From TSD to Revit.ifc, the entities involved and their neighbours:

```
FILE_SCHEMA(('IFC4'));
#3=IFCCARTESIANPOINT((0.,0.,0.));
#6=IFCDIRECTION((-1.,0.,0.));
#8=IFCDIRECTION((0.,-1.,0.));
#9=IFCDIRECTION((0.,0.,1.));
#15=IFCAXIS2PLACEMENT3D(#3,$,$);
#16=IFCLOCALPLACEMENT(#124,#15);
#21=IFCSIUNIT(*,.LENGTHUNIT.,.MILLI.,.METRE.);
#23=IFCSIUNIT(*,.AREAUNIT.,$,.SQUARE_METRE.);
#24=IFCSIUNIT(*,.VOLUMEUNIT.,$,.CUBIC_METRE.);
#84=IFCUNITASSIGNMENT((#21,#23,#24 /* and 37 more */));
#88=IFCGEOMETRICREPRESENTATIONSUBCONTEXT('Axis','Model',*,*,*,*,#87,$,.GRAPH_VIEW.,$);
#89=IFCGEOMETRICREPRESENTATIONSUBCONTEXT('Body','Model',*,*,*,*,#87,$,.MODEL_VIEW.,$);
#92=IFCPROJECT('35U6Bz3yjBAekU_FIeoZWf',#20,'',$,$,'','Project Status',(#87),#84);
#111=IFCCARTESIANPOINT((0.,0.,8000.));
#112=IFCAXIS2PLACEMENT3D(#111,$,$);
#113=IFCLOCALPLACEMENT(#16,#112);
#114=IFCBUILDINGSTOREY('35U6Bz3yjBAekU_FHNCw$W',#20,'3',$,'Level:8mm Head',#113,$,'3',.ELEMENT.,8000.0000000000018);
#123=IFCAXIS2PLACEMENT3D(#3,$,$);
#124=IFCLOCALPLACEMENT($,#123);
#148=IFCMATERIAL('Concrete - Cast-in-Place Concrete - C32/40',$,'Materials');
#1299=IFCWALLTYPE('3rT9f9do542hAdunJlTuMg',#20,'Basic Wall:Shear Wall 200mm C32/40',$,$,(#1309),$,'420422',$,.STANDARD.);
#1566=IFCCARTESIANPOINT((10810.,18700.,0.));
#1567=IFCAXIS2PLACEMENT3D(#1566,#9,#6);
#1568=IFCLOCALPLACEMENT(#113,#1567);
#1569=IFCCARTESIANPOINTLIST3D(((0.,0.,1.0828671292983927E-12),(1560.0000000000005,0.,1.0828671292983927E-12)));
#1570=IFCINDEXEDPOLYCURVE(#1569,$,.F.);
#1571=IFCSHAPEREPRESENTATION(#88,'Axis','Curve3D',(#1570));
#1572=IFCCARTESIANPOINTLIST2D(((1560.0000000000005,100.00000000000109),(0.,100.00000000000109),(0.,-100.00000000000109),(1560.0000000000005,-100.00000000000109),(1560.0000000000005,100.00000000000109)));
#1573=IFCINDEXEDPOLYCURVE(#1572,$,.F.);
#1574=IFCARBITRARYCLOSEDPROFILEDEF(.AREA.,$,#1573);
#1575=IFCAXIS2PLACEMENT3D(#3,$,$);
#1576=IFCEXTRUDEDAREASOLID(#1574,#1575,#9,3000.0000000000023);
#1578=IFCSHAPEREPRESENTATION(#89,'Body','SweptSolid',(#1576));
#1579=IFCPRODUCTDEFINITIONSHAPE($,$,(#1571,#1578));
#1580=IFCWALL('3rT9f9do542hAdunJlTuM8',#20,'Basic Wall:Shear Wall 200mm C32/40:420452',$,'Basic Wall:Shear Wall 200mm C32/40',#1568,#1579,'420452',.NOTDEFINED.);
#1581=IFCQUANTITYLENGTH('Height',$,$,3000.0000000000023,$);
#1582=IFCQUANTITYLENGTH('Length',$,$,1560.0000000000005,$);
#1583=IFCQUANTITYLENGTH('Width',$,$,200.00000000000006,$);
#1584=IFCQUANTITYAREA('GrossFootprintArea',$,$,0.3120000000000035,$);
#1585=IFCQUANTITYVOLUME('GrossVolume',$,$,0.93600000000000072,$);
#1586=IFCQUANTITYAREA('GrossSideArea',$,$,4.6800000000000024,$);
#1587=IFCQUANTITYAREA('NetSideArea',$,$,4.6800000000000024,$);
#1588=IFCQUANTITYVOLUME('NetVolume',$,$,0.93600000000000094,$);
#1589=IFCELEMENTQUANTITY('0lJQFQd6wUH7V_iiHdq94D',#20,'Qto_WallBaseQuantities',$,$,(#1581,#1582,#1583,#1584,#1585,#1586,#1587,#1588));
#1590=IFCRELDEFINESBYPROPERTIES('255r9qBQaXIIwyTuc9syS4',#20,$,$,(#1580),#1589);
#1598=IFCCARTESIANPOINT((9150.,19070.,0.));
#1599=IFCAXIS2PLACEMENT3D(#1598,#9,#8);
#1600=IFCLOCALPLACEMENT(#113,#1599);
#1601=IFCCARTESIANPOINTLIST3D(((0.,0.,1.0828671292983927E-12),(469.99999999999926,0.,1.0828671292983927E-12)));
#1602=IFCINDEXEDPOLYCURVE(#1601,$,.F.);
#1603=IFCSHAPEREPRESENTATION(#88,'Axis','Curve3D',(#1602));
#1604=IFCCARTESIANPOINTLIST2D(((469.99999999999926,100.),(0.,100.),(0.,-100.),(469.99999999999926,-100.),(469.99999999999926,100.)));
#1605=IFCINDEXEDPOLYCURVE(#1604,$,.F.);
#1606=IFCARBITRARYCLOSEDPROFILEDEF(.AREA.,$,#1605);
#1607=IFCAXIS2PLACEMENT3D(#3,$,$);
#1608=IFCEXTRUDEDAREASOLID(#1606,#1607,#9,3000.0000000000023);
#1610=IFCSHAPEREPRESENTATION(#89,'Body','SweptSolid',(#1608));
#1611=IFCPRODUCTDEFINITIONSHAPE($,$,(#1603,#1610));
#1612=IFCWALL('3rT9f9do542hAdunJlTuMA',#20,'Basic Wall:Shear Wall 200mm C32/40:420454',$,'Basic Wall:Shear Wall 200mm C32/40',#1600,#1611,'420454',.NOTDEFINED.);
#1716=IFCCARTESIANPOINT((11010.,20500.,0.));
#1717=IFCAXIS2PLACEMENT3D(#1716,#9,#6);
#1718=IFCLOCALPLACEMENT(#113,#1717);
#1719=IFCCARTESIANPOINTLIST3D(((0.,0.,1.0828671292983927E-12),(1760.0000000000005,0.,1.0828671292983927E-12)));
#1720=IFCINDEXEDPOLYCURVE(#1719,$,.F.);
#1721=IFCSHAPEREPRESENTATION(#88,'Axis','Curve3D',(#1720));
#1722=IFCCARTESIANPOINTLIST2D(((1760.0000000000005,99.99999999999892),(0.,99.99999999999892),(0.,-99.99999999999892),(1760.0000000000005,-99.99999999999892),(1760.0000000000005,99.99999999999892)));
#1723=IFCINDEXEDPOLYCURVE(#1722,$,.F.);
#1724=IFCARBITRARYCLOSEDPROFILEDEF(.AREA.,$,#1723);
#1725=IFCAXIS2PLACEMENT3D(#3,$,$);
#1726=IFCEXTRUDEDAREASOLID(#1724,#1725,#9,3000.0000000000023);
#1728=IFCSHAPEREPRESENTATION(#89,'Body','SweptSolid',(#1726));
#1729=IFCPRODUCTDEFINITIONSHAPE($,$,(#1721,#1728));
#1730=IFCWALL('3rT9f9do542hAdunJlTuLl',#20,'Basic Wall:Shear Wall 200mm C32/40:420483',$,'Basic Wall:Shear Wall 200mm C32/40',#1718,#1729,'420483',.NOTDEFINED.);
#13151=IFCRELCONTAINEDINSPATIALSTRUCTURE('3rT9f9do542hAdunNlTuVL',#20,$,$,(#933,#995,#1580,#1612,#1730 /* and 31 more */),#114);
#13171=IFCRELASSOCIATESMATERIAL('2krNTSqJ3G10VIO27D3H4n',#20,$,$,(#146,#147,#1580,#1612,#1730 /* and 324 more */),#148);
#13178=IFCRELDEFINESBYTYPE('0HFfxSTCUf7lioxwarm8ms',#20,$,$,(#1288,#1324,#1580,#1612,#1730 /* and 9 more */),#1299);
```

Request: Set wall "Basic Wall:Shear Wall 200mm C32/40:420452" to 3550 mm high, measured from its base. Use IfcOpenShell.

```python
import ifcopenshell
import ifcopenshell.api.pset
import ifcopenshell.geom
import ifcopenshell.util.element
import ifcopenshell.util.representation
import ifcopenshell.util.shape
import ifcopenshell.util.unit

model = ifcopenshell.open("TSD to Revit.ifc")
unit_scale = ifcopenshell.util.unit.calculate_unit_scale(model)
area_scale = ifcopenshell.util.unit.calculate_unit_scale(model, "AREAUNIT")
volume_scale = ifcopenshell.util.unit.calculate_unit_scale(model, "VOLUMEUNIT")
settings = ifcopenshell.geom.settings()


def volume(element):
    """Net volume in cubic metres, openings subtracted."""
    shape = ifcopenshell.geom.create_shape(settings, element)
    return ifcopenshell.util.shape.get_volume(shape.geometry)


wall = model.by_guid("3rT9f9do542hAdunJlTuM8")
before = volume(wall)

body = ifcopenshell.util.representation.get_representation(wall, "Model", "Body")
solid = body.Items[0]
old_height = solid.Depth
solid.Depth = 3.55 / unit_scale
after = volume(wall)
thickness = 0.2  # wall thickness in metres

# Update the stored height, areas and volumes.
qto = model.by_id(ifcopenshell.util.element.get_pset(wall, "Qto_WallBaseQuantities", should_inherit=False)["id"])
ifcopenshell.api.pset.edit_qto(model, qto=qto, properties={
    "Height": solid.Depth,
    "GrossVolume": ifcopenshell.util.element.get_pset(wall, "Qto_WallBaseQuantities", "GrossVolume") * solid.Depth / old_height,
    "GrossSideArea": ifcopenshell.util.element.get_pset(wall, "Qto_WallBaseQuantities", "GrossSideArea") * solid.Depth / old_height,
    "NetSideArea": after / thickness / area_scale,
    "NetVolume": after / volume_scale,
})

print(f"height {old_height:g} -> {solid.Depth:g}, volume {before:.3f} -> {after:.3f} m3")

model.write("TSD to Revit-out.ifc")
```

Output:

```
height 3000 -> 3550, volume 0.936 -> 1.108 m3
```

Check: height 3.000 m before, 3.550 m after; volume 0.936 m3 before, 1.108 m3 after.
